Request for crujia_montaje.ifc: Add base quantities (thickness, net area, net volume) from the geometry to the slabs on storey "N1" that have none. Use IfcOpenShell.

First a look at what the model holds.

```python
import ifcopenshell
import ifcopenshell.util.element
import ifcopenshell.util.unit

model = ifcopenshell.open("crujia_montaje.ifc")
print(model.schema)
for unit_type in ("LENGTHUNIT", "AREAUNIT", "VOLUMEUNIT"):
    print(unit_type, ifcopenshell.util.unit.calculate_unit_scale(model, unit_type))
storey = next(s for s in model.by_type("IfcBuildingStorey") if s.Name == "N1")
slabs = [e for e in ifcopenshell.util.element.get_decomposition(storey) if e.is_a("IfcSlab")]
for e in sorted(slabs, key=lambda e: e.id()):
    print(e.id(), e.is_a(), e.Name, list(ifcopenshell.util.element.get_psets(e, qtos_only=True)), sep=" | ")
```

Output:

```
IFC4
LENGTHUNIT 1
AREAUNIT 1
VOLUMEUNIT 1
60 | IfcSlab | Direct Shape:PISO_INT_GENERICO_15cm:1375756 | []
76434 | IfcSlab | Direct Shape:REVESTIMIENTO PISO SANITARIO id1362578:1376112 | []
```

```python
import ifcopenshell
import ifcopenshell.api.pset
import ifcopenshell.geom
import ifcopenshell.util.element
import ifcopenshell.util.shape
import ifcopenshell.util.unit

model = ifcopenshell.open("crujia_montaje.ifc")
unit_scale = ifcopenshell.util.unit.calculate_unit_scale(model)
area_scale = ifcopenshell.util.unit.calculate_unit_scale(model, "AREAUNIT")
volume_scale = ifcopenshell.util.unit.calculate_unit_scale(model, "VOLUMEUNIT")
settings = ifcopenshell.geom.settings()

storey = next(s for s in model.by_type("IfcBuildingStorey") if s.Name == "N1")
slabs = [e for e in ifcopenshell.util.element.get_decomposition(storey) if e.is_a("IfcSlab")]

for e in sorted(slabs, key=lambda e: e.id()):
    if ifcopenshell.util.element.get_psets(e, qtos_only=True, should_inherit=False):
        continue
    # Geometry comes back in metres, in the element's own axes.
    shape = ifcopenshell.geom.create_shape(settings, e)
    values = {
        "Width": ifcopenshell.util.shape.get_z(shape.geometry) / unit_scale,
        "NetArea": ifcopenshell.util.shape.get_footprint_area(shape.geometry) / area_scale,
        "NetVolume": ifcopenshell.util.shape.get_volume(shape.geometry) / volume_scale,
    }
    qto = ifcopenshell.api.pset.add_qto(model, product=e, name="Qto_SlabBaseQuantities")
    ifcopenshell.api.pset.edit_qto(model, qto=qto, properties=values)
    print(e.id(), {k: round(v, 3) for k, v in values.items()})

model.write("crujia_montaje_updated.ifc")
```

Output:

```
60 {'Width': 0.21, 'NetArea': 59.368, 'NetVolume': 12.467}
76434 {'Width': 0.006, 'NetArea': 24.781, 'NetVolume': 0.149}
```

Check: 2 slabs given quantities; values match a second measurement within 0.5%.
